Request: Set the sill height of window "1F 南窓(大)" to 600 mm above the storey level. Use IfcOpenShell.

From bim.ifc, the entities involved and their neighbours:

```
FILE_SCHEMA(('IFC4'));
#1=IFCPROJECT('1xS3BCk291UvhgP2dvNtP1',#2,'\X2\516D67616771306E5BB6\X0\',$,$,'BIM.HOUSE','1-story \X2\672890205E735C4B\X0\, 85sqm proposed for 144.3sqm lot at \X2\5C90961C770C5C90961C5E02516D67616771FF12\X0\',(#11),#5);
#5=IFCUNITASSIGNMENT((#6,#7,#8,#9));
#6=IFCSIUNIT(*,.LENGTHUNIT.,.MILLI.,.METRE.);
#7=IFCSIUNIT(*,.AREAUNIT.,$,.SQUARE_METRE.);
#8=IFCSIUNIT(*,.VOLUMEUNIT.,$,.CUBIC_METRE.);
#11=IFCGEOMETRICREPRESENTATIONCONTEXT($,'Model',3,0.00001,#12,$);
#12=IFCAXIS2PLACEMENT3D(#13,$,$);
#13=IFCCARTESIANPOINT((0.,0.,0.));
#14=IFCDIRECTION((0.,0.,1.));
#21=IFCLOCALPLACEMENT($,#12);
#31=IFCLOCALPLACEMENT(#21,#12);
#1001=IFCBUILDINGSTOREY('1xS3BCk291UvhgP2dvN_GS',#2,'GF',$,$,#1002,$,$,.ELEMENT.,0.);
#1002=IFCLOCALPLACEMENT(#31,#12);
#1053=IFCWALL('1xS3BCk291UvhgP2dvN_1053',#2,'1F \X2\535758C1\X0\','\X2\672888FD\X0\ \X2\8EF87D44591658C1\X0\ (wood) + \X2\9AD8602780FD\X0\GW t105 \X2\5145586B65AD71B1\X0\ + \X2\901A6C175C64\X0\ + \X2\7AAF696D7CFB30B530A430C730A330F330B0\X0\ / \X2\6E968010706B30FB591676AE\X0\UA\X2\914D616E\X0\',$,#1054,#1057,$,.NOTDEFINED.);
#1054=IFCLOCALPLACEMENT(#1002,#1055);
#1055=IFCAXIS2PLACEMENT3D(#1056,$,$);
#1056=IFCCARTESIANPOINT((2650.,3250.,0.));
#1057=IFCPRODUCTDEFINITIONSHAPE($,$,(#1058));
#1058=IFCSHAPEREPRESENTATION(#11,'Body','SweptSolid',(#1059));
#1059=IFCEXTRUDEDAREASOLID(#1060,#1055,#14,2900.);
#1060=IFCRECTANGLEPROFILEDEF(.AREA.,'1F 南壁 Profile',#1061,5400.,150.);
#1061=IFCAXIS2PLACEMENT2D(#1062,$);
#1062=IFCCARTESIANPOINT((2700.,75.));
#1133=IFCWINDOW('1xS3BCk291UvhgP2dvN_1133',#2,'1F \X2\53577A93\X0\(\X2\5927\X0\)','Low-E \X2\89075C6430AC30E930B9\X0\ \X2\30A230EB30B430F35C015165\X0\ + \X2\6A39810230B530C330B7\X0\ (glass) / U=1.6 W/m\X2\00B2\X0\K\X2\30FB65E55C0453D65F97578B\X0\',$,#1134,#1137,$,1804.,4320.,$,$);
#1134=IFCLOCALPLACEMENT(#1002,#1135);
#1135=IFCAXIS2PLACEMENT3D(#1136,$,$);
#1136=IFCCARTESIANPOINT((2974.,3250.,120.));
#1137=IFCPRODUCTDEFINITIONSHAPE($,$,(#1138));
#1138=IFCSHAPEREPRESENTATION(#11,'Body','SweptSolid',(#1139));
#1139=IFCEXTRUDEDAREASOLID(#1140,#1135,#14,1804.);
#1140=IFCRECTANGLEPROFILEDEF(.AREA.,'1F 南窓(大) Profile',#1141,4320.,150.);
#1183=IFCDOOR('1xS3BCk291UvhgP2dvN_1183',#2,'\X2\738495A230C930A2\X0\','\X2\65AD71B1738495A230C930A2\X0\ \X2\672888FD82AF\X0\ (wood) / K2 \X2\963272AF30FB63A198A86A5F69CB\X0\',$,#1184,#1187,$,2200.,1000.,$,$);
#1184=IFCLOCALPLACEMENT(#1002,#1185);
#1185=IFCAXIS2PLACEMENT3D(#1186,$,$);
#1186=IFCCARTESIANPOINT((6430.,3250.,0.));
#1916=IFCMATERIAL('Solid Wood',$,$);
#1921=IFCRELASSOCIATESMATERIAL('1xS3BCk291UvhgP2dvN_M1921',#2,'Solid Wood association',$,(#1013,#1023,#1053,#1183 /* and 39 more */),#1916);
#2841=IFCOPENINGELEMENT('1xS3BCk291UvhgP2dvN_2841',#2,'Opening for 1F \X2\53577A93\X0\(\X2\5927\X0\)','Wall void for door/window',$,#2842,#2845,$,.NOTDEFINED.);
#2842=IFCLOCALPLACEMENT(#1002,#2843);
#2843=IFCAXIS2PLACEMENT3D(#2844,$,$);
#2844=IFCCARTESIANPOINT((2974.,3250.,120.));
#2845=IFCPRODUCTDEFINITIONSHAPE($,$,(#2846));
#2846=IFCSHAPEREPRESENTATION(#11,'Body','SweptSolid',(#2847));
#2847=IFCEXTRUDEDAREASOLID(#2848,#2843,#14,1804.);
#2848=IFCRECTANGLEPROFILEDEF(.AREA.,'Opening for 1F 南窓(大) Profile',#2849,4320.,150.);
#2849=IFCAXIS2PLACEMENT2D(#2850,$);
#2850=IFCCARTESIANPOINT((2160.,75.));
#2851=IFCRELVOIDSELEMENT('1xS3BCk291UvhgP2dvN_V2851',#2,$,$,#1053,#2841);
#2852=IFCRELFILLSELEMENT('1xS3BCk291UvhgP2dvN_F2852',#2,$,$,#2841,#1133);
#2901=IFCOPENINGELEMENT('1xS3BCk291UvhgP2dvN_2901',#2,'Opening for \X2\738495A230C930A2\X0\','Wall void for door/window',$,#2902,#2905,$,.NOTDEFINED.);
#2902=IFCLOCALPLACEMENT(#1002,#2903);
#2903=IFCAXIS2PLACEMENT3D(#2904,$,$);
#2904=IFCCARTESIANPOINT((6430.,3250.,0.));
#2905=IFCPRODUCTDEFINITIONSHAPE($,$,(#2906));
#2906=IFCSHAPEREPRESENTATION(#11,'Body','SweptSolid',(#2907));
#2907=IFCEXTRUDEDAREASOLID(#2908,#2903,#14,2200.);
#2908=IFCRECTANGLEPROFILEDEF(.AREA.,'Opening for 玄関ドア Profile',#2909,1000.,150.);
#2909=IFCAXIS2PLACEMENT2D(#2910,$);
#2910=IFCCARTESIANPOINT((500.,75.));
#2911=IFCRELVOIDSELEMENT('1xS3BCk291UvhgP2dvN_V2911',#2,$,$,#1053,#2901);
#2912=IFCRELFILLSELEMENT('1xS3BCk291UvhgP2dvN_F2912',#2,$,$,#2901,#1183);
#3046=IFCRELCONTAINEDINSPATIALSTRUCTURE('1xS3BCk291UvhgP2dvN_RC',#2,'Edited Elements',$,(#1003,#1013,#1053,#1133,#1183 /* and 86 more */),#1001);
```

```python
import numpy as np
import ifcopenshell
import ifcopenshell.api.geometry
import ifcopenshell.geom
import ifcopenshell.util.element
import ifcopenshell.util.placement
import ifcopenshell.util.shape
import ifcopenshell.util.unit

model = ifcopenshell.open("bim.ifc")
unit_scale = ifcopenshell.util.unit.calculate_unit_scale(model)

window = model.by_guid("1xS3BCk291UvhgP2dvN_1133")
opening = window.FillsVoids[0].RelatingOpeningElement
storey = ifcopenshell.util.element.get_container(window, ifc_class="IfcBuildingStorey")
level = ifcopenshell.util.placement.get_local_placement(storey.ObjectPlacement)[2, 3]

# The opening's origin need not be at the sill, so measure its lowest point.
shape = ifcopenshell.geom.create_shape(ifcopenshell.geom.settings(), opening)
bottom = ifcopenshell.util.shape.get_shape_bottom_elevation(shape, shape.geometry) / unit_scale
dz = level + 0.6 / unit_scale - bottom

shift = np.array([0.0, 0.0, dz])
# The window is not placed relative to its opening, so move both.
for product in (opening, window):
    matrix = ifcopenshell.util.placement.get_local_placement(product.ObjectPlacement)
    matrix[:3, 3] += shift
    ifcopenshell.api.geometry.edit_object_placement(model, product=product, matrix=matrix, is_si=False)

print(f"moved by {dz * unit_scale:+.3f} m")

model.write("bim_rev.ifc")
```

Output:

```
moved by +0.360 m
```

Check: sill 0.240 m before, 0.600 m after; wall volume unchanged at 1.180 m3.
